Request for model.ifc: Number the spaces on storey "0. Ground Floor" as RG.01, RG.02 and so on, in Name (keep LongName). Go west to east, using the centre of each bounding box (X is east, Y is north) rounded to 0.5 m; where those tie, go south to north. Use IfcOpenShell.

First a look at what the model holds.

```python
import ifcopenshell
import ifcopenshell.util.element
import ifcopenshell.util.placement

model = ifcopenshell.open("model.ifc")
print(model.schema)
storey = next(s for s in model.by_type("IfcBuildingStorey") if s.Name == "0. Ground Floor")
spaces = [e for e in ifcopenshell.util.element.get_decomposition(storey) if e.is_a("IfcSpace")]
for e in sorted(spaces, key=lambda e: e.id()):
    origin = ifcopenshell.util.placement.get_local_placement(e.ObjectPlacement)[:3, 3]
    print(e.id(), e.Name, e.LongName, origin.round(2) + 0.0, sep=" | ")
```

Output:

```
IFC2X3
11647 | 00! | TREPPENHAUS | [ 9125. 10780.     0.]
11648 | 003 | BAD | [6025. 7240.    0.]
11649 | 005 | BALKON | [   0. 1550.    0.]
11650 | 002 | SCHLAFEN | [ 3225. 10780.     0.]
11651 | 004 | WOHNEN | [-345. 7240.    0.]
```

```python
import ifcopenshell
import ifcopenshell.geom
import ifcopenshell.util.element
import ifcopenshell.util.shape

model = ifcopenshell.open("model.ifc")
settings = ifcopenshell.geom.settings()
settings.set("use-world-coords", True)


def centre(element):
    shape = ifcopenshell.geom.create_shape(settings, element)
    return ifcopenshell.util.shape.get_bbox_centroid(shape.geometry)


storey = next(s for s in model.by_type("IfcBuildingStorey") if s.Name == "0. Ground Floor")
spaces = [e for e in ifcopenshell.util.element.get_decomposition(storey) if e.is_a("IfcSpace")]

# Insertion points can sit at a corner or the storey origin, so sort by the geometry (in metres).
centres = {e: centre(e) for e in spaces}
spaces.sort(key=lambda e: (round(centres[e][0] / 0.5), centres[e][1]))

for i, e in enumerate(spaces, start=1):
    number = f"RG.{i:02d}"
    e.Name = number
    print(e.id(), number)

model.write("model_edited.ifc")
```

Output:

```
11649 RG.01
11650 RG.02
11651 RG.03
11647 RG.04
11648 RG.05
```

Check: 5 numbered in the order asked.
